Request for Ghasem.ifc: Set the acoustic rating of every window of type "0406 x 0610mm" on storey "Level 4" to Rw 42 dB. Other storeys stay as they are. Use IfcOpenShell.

First a look at what the model holds.

```python
import ifcopenshell
import ifcopenshell.util.element

model = ifcopenshell.open("Ghasem.ifc")
print(model.schema)
storey = next(s for s in model.by_type("IfcBuildingStorey") if s.Name == "Level 4")
windows = [e for e in ifcopenshell.util.element.get_decomposition(storey) if e.is_a("IfcWindow")]
seen = {}
for e in windows:
    element_type = ifcopenshell.util.element.get_type(e)
    key = (element_type.Name if element_type != e and element_type else None, ifcopenshell.util.element.get_pset(e, "Pset_WindowCommon", "AcousticRating"))
    seen[key] = seen.get(key, 0) + 1
for (name, value), count in sorted(seen.items(), key=str):
    print(count, "x", name, "|", value)
```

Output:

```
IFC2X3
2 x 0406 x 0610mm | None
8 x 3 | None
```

```python
import ifcopenshell
import ifcopenshell.api.pset
import ifcopenshell.util.element

model = ifcopenshell.open("Ghasem.ifc")

storey = next(s for s in model.by_type("IfcBuildingStorey") if s.Name == "Level 4")
windows = [e for e in ifcopenshell.util.element.get_decomposition(storey) if e.is_a("IfcWindow")]

count = 0
for e in windows:
    element_type = ifcopenshell.util.element.get_type(e)
    if element_type in (None, e) or element_type.Name != "0406 x 0610mm":
        continue
    # add_pset returns the element's existing set when there is one.
    pset = ifcopenshell.api.pset.add_pset(model, product=e, name="Pset_WindowCommon")
    ifcopenshell.api.pset.edit_pset(model, pset=pset, properties={"AcousticRating": "Rw 42 dB"})
    count += 1

print(count, "windows updated")

model.write("Ghasem-out.ifc")
```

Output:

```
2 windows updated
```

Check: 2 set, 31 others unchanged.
